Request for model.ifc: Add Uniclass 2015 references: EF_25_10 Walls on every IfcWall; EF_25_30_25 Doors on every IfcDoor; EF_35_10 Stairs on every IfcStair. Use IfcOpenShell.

First a look at what the model holds.

```python
import ifcopenshell

model = ifcopenshell.open("model.ifc")
print(model.schema)
print("classifications:", [c.Name for c in model.by_type("IfcClassification")])
for ifc_class in ("IfcDoor", "IfcRoof", "IfcStair", "IfcWall", "IfcWindow"):
    print(ifc_class, len(model.by_type(ifc_class)))
```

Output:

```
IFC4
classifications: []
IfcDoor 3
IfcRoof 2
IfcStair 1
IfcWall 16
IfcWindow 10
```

```python
import ifcopenshell
import ifcopenshell.api.classification

model = ifcopenshell.open("model.ifc")

system = ifcopenshell.api.classification.add_classification(model, classification="Uniclass 2015")

codes = {
    "IfcWall": ("EF_25_10", "Walls"),
    "IfcDoor": ("EF_25_30_25", "Doors"),
    "IfcStair": ("EF_35_10", "Stairs"),
}
for ifc_class, (code, name) in codes.items():
    products = model.by_type(ifc_class)
    ifcopenshell.api.classification.add_reference(
        model, products=products, classification=system, identification=code, name=name
    )
    print(code, len(products))

model.write("model_v2.ifc")
```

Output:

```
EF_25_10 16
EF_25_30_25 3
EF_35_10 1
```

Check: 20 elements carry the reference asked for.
